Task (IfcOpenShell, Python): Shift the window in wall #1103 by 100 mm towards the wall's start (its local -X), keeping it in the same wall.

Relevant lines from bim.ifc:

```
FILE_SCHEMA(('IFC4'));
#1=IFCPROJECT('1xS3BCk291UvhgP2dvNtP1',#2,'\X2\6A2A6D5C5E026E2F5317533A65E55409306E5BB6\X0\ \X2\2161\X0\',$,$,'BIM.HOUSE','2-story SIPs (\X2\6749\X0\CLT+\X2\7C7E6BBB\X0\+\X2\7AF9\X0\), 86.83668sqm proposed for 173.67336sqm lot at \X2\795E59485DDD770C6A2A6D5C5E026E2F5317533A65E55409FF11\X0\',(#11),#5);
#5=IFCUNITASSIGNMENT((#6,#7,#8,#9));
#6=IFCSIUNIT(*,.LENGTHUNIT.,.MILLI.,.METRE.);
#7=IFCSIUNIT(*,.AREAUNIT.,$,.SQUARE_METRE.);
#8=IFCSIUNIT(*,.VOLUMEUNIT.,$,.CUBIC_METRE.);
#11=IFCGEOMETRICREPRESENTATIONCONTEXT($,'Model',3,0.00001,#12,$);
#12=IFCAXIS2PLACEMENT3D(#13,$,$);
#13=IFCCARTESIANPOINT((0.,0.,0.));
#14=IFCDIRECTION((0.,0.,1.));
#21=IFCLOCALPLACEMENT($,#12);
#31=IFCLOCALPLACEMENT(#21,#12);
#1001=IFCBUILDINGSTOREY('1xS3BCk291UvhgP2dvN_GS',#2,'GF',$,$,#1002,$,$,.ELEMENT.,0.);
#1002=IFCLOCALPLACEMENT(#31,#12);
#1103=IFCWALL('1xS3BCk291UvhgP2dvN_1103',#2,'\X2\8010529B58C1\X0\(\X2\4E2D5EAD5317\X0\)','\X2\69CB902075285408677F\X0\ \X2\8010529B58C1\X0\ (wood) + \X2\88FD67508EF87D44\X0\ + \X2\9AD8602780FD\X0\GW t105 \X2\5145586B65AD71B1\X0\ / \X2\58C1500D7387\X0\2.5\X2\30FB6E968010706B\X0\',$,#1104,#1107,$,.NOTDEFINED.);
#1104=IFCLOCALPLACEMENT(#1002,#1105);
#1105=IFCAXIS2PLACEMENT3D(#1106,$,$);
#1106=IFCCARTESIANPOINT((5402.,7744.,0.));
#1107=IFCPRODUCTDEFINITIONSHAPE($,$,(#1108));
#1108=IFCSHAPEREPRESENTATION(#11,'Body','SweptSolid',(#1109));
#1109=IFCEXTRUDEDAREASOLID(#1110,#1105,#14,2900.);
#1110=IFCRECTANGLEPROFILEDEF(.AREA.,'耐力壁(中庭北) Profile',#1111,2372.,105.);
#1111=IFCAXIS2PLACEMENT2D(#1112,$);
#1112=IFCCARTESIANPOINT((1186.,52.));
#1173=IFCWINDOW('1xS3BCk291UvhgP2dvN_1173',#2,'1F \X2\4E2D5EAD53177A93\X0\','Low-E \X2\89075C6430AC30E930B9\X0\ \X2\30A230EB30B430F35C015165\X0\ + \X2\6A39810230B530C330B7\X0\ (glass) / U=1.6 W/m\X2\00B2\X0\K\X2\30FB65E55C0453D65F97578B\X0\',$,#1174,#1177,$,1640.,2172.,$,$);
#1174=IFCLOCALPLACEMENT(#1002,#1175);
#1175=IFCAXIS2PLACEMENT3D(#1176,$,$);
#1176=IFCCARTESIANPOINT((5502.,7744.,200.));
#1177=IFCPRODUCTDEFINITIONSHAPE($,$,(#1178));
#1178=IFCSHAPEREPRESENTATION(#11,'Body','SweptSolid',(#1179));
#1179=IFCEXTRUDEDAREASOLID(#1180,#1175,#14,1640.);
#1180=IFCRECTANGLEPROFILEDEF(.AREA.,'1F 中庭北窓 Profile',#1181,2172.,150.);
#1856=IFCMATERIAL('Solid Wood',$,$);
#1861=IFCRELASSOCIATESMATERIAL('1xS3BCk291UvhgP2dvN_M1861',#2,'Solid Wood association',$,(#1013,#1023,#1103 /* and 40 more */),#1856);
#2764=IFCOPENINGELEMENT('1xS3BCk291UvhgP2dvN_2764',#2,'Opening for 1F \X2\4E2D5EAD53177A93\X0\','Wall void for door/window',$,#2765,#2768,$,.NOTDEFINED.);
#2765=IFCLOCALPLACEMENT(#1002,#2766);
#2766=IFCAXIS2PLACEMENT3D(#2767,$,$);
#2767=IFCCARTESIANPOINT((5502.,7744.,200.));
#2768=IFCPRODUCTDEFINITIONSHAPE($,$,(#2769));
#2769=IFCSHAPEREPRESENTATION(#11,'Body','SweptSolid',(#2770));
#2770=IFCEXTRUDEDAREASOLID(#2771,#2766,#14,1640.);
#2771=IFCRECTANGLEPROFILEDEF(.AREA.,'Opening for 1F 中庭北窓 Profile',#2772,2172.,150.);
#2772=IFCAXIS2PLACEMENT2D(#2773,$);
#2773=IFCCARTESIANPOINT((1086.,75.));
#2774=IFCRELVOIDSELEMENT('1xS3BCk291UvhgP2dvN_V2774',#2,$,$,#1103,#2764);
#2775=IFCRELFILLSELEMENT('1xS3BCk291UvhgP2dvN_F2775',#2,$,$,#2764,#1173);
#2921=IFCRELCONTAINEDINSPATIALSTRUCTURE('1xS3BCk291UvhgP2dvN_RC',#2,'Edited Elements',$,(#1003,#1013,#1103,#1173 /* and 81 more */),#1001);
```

```python
import ifcopenshell
import ifcopenshell.api.geometry
import ifcopenshell.util.placement
import ifcopenshell.util.unit

model = ifcopenshell.open("bim.ifc")
unit_scale = ifcopenshell.util.unit.calculate_unit_scale(model)

window = model.by_guid("1xS3BCk291UvhgP2dvN_1173")
opening = window.FillsVoids[0].RelatingOpeningElement
wall = opening.VoidsElements[0].RelatingBuildingElement

wall_matrix = ifcopenshell.util.placement.get_local_placement(wall.ObjectPlacement)
shift = wall_matrix[:3, 0] * -0.1 / unit_scale
before = ifcopenshell.util.placement.get_local_placement(window.ObjectPlacement)[:3, 3].copy()

# The window is not placed relative to its opening, so move both.
for product in (opening, window):
    matrix = ifcopenshell.util.placement.get_local_placement(product.ObjectPlacement)
    matrix[:3, 3] += shift
    ifcopenshell.api.geometry.edit_object_placement(model, product=product, matrix=matrix, is_si=False)

after = ifcopenshell.util.placement.get_local_placement(window.ObjectPlacement)[:3, 3]
print("window moved by", (after - before).round(3) + 0.0)

model.write("bim-out.ifc")
```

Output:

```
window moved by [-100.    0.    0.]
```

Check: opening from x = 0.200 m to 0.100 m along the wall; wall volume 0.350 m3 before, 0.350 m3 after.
